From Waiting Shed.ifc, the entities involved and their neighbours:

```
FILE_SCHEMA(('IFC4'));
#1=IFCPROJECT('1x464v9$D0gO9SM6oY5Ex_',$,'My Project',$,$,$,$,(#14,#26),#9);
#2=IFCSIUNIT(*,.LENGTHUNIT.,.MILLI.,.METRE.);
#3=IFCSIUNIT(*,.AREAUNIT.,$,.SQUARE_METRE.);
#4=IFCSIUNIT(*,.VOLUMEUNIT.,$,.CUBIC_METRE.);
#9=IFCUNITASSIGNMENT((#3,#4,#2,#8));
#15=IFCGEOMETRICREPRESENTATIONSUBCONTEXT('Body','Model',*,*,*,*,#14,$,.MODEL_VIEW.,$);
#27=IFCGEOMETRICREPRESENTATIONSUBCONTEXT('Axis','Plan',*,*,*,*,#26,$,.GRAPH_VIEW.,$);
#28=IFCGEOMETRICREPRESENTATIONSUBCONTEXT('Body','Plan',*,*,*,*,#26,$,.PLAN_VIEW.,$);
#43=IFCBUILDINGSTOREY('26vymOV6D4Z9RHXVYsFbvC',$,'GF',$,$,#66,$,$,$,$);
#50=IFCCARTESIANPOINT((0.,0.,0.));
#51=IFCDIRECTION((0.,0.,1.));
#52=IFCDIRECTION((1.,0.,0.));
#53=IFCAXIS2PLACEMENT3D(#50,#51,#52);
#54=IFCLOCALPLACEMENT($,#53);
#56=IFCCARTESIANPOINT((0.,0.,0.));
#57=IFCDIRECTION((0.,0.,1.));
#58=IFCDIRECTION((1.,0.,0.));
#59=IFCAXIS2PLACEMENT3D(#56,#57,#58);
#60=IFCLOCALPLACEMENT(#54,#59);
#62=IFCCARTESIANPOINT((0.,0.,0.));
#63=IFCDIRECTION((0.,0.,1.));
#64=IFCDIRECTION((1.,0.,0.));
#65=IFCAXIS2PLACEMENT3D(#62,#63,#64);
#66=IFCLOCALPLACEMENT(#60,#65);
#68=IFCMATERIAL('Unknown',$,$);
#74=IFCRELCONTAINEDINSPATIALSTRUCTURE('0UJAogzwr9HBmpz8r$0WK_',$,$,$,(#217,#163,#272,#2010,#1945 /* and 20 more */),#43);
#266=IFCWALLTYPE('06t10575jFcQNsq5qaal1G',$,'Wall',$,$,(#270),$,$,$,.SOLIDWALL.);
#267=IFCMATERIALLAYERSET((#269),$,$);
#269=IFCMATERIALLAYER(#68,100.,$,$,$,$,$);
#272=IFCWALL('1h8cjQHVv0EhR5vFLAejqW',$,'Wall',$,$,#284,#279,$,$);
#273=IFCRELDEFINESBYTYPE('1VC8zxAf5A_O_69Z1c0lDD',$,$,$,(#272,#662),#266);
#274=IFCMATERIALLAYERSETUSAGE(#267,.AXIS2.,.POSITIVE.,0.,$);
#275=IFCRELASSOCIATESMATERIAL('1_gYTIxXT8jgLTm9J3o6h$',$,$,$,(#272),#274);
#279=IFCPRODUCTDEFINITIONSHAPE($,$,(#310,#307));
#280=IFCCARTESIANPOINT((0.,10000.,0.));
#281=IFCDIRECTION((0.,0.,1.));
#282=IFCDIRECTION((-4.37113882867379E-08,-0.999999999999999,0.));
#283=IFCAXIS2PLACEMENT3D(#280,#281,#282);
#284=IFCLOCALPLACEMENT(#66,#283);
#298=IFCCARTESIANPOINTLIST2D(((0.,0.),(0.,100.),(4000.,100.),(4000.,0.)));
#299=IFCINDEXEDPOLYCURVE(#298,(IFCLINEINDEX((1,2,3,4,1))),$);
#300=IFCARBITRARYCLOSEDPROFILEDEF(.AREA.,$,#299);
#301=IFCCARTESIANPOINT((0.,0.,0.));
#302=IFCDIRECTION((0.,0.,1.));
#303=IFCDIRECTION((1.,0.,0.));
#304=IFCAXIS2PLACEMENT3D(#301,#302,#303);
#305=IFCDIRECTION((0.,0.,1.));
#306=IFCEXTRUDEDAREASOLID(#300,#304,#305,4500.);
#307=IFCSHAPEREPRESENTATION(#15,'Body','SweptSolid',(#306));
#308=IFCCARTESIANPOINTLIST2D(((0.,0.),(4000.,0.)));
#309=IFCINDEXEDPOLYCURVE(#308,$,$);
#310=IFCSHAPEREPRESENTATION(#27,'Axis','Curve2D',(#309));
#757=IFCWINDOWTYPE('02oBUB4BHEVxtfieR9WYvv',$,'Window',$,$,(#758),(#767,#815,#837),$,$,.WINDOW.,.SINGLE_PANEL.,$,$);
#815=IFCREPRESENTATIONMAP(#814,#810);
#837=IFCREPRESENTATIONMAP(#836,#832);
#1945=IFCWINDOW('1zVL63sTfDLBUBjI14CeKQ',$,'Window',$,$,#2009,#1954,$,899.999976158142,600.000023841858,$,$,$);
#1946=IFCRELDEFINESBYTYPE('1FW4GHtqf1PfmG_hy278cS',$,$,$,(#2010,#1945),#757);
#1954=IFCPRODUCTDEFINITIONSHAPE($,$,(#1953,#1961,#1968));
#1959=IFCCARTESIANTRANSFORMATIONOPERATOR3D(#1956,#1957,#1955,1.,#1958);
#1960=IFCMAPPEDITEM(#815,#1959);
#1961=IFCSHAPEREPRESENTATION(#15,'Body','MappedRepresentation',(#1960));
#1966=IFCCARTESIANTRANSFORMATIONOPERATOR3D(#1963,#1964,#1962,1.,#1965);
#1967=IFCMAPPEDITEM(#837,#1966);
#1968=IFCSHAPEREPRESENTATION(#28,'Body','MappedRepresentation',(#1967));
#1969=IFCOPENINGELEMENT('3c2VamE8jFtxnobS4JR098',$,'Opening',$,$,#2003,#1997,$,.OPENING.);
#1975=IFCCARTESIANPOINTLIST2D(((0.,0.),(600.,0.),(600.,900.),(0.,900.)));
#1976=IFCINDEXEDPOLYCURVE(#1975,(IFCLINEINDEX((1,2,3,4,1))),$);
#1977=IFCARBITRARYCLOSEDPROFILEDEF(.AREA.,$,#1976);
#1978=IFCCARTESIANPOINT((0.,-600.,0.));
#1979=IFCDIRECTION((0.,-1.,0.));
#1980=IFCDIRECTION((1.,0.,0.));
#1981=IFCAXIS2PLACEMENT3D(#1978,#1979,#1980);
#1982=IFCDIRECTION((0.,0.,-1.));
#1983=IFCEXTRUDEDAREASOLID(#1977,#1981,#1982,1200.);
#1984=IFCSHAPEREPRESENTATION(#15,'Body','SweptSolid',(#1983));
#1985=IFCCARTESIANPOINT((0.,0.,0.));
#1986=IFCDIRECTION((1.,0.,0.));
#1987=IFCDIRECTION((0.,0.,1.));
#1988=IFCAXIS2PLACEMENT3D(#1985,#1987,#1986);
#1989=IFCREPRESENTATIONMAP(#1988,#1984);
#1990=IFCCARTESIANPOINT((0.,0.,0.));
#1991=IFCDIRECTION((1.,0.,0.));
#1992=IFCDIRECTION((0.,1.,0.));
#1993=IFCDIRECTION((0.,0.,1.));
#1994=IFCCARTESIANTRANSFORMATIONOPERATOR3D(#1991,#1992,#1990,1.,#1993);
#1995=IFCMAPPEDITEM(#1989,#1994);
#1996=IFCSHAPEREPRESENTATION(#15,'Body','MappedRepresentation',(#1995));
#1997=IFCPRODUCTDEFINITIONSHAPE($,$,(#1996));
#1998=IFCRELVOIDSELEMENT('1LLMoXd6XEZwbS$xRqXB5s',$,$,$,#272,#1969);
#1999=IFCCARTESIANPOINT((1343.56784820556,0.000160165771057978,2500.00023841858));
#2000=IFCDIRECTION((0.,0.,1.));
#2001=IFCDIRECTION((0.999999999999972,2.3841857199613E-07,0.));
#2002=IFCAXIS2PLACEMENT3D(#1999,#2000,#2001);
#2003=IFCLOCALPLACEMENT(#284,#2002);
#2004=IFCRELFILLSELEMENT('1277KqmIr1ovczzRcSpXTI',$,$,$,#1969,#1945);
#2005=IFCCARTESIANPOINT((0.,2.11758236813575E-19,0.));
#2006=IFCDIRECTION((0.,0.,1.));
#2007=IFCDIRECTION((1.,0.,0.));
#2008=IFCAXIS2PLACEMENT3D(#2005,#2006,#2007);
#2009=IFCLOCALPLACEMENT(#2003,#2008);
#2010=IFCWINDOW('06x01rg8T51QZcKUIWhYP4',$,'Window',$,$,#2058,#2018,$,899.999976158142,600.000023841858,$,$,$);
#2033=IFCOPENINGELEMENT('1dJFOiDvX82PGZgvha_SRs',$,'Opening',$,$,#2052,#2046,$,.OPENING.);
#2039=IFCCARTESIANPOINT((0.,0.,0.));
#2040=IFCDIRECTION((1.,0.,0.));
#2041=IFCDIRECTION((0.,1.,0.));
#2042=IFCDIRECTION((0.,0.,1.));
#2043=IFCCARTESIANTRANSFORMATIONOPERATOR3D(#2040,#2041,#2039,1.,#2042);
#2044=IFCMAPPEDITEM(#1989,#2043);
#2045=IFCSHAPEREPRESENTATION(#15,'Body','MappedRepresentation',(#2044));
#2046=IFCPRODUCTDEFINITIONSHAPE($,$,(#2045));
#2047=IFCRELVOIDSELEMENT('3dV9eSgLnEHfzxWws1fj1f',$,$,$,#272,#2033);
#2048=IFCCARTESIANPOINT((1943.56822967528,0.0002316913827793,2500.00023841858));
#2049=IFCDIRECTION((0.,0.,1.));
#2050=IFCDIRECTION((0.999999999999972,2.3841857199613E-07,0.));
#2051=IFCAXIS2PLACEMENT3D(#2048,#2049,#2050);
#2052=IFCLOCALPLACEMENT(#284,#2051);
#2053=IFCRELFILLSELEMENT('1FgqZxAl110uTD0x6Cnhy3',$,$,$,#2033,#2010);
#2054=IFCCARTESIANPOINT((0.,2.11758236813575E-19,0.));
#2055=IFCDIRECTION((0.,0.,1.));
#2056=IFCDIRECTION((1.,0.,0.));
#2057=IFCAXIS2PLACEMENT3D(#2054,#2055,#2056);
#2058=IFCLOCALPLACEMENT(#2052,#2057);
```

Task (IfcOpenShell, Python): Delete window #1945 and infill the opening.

```python
import ifcopenshell
import ifcopenshell.api.feature
import ifcopenshell.api.root
import ifcopenshell.geom
import ifcopenshell.util.shape

model = ifcopenshell.open("Waiting Shed.ifc")
settings = ifcopenshell.geom.settings()


def volume(element):
    """Net volume in cubic metres, openings subtracted."""
    shape = ifcopenshell.geom.create_shape(settings, element)
    return ifcopenshell.util.shape.get_volume(shape.geometry)


window = model.by_id(1945)
opening = window.FillsVoids[0].RelatingOpeningElement
wall = opening.VoidsElements[0].RelatingBuildingElement
before = volume(wall)

ifcopenshell.api.root.remove_product(model, product=window)
ifcopenshell.api.feature.remove_feature(model, feature=opening)

after = volume(wall)

print(f"wall volume {before:.3f} -> {after:.3f} m3")

model.write("Waiting Shed_edited.ifc")
```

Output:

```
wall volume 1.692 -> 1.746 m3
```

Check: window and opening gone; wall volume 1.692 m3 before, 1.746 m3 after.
